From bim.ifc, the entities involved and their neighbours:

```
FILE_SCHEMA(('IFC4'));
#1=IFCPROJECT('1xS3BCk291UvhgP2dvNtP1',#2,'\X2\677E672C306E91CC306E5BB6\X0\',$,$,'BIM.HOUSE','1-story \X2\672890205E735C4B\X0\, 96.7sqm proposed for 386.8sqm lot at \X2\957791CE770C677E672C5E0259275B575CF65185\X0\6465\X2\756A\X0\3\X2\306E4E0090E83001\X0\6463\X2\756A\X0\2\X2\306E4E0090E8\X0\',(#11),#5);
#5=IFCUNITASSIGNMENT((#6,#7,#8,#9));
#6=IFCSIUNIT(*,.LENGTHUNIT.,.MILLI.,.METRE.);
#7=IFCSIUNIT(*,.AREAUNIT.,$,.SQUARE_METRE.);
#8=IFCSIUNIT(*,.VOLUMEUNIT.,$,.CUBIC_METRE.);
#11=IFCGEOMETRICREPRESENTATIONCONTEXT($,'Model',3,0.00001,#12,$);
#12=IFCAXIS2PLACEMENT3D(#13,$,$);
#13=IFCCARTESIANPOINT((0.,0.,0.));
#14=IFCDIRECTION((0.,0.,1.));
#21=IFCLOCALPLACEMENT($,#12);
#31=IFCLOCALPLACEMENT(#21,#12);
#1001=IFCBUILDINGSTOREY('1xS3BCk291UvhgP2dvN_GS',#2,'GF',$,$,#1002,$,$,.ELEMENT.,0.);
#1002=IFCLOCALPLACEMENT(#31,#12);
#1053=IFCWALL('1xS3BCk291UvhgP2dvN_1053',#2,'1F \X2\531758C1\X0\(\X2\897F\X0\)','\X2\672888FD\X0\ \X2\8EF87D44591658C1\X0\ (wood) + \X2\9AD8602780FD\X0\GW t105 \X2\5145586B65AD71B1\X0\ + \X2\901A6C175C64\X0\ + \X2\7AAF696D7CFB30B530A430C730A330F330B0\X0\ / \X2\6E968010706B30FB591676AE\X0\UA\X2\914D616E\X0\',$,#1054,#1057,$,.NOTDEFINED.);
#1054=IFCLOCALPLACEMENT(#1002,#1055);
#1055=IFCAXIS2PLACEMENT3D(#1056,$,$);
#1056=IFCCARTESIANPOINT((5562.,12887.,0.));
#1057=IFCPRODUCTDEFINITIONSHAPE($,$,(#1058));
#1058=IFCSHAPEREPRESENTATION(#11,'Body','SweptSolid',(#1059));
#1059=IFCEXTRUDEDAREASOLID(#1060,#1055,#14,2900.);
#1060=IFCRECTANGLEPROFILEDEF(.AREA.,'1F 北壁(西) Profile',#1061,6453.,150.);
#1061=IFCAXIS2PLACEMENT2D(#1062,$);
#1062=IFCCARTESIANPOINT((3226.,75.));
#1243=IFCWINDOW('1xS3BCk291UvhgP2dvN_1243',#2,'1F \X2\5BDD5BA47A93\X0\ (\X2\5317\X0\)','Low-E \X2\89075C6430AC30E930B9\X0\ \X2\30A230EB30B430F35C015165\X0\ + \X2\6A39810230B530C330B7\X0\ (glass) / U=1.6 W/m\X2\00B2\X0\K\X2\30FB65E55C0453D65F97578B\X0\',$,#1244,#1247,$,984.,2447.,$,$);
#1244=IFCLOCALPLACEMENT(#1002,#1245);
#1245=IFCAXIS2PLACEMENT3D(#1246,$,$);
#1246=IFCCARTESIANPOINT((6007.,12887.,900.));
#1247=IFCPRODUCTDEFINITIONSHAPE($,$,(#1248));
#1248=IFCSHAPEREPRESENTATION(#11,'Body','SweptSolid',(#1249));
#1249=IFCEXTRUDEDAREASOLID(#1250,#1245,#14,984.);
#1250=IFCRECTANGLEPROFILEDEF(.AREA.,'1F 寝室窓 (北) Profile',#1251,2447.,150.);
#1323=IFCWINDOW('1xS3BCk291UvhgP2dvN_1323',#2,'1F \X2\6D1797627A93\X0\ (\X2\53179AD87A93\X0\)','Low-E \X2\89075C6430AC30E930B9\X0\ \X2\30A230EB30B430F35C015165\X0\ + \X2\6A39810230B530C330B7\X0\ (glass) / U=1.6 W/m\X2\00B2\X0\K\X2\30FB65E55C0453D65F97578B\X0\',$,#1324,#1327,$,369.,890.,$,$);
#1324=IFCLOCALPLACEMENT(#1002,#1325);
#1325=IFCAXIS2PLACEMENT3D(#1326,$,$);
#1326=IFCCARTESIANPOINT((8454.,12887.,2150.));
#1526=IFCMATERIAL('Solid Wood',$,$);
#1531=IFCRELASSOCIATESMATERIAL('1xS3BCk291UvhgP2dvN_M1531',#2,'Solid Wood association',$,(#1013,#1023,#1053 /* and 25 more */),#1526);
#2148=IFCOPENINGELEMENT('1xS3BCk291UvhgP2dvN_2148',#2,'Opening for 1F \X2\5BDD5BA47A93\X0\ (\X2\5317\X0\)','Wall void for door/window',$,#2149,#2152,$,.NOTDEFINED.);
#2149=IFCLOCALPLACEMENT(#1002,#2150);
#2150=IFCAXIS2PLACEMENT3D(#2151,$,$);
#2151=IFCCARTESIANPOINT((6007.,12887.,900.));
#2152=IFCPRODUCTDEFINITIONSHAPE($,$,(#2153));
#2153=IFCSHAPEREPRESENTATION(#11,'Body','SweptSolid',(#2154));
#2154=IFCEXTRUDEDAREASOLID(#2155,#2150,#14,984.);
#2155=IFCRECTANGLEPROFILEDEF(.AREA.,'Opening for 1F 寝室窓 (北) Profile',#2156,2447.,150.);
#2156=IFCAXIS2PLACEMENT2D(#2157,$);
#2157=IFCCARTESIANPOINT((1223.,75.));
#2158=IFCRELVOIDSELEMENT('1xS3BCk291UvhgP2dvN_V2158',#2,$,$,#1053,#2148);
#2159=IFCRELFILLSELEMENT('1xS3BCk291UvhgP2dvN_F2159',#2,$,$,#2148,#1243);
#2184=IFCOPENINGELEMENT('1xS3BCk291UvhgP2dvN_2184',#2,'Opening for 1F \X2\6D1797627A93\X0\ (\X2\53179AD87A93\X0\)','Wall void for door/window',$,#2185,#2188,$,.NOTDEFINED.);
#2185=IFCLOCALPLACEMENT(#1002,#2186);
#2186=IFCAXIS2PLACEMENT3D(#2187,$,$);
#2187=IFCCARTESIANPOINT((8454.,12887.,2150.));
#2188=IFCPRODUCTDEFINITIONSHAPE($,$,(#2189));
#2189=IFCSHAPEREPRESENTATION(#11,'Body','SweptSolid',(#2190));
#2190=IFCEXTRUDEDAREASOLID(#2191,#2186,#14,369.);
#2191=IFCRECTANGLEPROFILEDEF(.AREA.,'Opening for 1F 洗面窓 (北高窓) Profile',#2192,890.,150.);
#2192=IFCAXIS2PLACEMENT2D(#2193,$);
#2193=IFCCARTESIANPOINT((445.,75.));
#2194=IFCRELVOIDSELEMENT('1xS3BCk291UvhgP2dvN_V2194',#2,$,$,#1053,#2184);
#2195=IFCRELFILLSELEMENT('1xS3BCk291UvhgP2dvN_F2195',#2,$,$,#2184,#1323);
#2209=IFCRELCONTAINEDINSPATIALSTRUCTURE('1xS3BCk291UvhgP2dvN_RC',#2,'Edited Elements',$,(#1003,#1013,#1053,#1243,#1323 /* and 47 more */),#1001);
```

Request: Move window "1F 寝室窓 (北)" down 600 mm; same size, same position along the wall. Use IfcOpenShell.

```python
import numpy as np
import ifcopenshell
import ifcopenshell.api.geometry
import ifcopenshell.util.placement
import ifcopenshell.util.unit

model = ifcopenshell.open("bim.ifc")
unit_scale = ifcopenshell.util.unit.calculate_unit_scale(model)

window = model.by_guid("1xS3BCk291UvhgP2dvN_1243")
opening = window.FillsVoids[0].RelatingOpeningElement
dz = -600.0

shift = np.array([0.0, 0.0, dz])
# The window is not placed relative to its opening, so move both.
for product in (opening, window):
    matrix = ifcopenshell.util.placement.get_local_placement(product.ObjectPlacement)
    matrix[:3, 3] += shift
    ifcopenshell.api.geometry.edit_object_placement(model, product=product, matrix=matrix, is_si=False)

print(f"moved by {dz * unit_scale:+.3f} m")

model.write("bim_v2.ifc")
```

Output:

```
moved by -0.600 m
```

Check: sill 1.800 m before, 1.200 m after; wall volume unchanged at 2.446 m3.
